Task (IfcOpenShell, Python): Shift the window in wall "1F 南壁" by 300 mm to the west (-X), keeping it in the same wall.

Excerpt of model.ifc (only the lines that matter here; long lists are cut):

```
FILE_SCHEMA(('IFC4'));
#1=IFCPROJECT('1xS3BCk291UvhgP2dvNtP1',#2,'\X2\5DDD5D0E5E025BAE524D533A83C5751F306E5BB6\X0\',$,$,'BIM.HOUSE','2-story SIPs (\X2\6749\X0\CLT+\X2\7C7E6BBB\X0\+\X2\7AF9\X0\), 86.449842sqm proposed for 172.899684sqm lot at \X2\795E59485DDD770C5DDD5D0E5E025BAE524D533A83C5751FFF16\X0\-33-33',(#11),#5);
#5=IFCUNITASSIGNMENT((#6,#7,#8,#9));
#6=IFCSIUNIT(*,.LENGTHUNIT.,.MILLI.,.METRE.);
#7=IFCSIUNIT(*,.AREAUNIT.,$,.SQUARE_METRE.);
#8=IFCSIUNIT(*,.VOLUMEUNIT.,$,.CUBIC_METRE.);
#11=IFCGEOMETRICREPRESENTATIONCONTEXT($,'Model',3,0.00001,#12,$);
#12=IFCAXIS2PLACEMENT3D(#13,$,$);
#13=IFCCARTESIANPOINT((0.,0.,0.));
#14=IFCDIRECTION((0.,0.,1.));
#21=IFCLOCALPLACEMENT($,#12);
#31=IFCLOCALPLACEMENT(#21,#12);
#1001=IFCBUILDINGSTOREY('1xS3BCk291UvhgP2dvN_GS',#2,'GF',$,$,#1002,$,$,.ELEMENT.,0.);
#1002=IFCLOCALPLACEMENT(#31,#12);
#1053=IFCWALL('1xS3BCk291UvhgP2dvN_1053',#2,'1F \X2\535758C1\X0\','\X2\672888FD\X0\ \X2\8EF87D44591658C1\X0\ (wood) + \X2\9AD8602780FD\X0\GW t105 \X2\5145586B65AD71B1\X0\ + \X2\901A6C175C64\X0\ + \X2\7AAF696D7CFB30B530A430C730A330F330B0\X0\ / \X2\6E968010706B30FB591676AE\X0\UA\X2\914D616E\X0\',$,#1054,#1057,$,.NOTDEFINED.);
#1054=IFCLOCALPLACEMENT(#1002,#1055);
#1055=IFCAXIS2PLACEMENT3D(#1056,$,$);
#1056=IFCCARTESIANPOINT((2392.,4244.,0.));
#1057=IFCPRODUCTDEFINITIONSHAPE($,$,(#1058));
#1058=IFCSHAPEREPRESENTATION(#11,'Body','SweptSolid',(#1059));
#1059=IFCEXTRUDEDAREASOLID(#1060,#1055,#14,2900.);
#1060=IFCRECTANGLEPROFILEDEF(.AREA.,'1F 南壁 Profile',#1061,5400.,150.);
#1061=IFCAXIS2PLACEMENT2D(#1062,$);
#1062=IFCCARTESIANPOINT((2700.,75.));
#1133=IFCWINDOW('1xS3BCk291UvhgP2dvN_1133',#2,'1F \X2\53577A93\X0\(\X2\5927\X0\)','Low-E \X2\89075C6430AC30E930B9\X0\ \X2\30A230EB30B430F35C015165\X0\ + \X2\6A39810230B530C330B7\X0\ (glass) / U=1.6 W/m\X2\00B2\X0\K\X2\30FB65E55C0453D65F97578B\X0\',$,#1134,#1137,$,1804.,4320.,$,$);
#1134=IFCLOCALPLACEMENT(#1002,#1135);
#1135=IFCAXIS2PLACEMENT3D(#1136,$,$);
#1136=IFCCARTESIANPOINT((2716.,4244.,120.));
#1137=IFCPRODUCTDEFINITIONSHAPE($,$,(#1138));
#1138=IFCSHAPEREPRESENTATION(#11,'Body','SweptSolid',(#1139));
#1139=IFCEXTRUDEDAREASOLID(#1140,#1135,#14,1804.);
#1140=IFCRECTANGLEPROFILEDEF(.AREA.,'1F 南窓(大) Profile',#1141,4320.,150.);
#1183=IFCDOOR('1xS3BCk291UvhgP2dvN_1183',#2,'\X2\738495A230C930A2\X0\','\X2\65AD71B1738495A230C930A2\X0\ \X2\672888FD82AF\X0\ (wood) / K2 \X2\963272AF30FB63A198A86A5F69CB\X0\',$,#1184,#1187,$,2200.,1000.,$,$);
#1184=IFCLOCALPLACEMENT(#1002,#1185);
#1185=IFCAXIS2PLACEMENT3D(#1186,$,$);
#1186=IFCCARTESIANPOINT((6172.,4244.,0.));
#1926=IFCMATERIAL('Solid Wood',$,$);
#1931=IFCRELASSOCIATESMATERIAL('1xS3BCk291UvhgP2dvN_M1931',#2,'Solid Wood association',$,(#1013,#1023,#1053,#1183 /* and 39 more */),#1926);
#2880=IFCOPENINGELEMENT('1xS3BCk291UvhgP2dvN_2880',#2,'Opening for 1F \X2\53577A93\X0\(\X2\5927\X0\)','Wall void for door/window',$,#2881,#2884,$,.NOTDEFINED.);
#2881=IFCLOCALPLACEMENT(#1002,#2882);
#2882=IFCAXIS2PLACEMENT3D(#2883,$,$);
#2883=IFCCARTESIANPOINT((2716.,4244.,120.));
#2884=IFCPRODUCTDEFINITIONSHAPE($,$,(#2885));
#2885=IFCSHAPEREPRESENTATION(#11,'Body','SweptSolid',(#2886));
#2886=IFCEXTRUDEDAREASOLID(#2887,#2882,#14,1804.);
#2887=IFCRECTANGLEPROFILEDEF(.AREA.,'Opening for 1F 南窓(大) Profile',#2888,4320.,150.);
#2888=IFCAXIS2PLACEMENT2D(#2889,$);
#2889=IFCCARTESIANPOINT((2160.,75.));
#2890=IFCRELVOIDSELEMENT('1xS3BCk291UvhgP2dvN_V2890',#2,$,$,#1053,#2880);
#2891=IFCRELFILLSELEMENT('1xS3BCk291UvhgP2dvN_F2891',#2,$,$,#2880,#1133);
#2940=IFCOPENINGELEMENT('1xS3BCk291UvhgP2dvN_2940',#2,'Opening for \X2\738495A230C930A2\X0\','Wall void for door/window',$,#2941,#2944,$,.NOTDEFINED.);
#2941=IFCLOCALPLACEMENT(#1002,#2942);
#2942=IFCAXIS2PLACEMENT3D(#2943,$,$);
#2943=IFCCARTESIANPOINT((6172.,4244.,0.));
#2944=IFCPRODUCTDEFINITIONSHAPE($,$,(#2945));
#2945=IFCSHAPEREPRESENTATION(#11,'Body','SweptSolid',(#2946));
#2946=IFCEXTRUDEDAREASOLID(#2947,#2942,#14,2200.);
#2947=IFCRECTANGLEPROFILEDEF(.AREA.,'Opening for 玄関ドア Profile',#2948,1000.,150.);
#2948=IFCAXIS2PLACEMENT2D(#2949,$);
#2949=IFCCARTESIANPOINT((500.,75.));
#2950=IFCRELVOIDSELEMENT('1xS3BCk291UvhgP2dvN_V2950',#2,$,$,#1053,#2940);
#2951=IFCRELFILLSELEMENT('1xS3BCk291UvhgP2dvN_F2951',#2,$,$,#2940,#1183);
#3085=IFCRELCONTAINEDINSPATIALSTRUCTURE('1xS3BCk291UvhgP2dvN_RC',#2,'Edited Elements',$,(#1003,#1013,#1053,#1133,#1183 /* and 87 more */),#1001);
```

```python
import ifcopenshell
import ifcopenshell.api.geometry
import ifcopenshell.util.placement
import ifcopenshell.util.unit

model = ifcopenshell.open("model.ifc")
unit_scale = ifcopenshell.util.unit.calculate_unit_scale(model)

window = model.by_guid("1xS3BCk291UvhgP2dvN_1133")
opening = window.FillsVoids[0].RelatingOpeningElement
wall = opening.VoidsElements[0].RelatingBuildingElement

wall_matrix = ifcopenshell.util.placement.get_local_placement(wall.ObjectPlacement)
shift = wall_matrix[:3, 0] * -0.3 / unit_scale
before = ifcopenshell.util.placement.get_local_placement(window.ObjectPlacement)[:3, 3].copy()

# The window is not placed relative to its opening, so move both.
for product in (opening, window):
    matrix = ifcopenshell.util.placement.get_local_placement(product.ObjectPlacement)
    matrix[:3, 3] += shift
    ifcopenshell.api.geometry.edit_object_placement(model, product=product, matrix=matrix, is_si=False)

after = ifcopenshell.util.placement.get_local_placement(window.ObjectPlacement)[:3, 3]
print("window moved by", (after - before).round(3) + 0.0)

model.write("model-out.ifc")
```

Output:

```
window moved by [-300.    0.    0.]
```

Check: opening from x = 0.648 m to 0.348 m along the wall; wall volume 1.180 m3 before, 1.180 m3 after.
